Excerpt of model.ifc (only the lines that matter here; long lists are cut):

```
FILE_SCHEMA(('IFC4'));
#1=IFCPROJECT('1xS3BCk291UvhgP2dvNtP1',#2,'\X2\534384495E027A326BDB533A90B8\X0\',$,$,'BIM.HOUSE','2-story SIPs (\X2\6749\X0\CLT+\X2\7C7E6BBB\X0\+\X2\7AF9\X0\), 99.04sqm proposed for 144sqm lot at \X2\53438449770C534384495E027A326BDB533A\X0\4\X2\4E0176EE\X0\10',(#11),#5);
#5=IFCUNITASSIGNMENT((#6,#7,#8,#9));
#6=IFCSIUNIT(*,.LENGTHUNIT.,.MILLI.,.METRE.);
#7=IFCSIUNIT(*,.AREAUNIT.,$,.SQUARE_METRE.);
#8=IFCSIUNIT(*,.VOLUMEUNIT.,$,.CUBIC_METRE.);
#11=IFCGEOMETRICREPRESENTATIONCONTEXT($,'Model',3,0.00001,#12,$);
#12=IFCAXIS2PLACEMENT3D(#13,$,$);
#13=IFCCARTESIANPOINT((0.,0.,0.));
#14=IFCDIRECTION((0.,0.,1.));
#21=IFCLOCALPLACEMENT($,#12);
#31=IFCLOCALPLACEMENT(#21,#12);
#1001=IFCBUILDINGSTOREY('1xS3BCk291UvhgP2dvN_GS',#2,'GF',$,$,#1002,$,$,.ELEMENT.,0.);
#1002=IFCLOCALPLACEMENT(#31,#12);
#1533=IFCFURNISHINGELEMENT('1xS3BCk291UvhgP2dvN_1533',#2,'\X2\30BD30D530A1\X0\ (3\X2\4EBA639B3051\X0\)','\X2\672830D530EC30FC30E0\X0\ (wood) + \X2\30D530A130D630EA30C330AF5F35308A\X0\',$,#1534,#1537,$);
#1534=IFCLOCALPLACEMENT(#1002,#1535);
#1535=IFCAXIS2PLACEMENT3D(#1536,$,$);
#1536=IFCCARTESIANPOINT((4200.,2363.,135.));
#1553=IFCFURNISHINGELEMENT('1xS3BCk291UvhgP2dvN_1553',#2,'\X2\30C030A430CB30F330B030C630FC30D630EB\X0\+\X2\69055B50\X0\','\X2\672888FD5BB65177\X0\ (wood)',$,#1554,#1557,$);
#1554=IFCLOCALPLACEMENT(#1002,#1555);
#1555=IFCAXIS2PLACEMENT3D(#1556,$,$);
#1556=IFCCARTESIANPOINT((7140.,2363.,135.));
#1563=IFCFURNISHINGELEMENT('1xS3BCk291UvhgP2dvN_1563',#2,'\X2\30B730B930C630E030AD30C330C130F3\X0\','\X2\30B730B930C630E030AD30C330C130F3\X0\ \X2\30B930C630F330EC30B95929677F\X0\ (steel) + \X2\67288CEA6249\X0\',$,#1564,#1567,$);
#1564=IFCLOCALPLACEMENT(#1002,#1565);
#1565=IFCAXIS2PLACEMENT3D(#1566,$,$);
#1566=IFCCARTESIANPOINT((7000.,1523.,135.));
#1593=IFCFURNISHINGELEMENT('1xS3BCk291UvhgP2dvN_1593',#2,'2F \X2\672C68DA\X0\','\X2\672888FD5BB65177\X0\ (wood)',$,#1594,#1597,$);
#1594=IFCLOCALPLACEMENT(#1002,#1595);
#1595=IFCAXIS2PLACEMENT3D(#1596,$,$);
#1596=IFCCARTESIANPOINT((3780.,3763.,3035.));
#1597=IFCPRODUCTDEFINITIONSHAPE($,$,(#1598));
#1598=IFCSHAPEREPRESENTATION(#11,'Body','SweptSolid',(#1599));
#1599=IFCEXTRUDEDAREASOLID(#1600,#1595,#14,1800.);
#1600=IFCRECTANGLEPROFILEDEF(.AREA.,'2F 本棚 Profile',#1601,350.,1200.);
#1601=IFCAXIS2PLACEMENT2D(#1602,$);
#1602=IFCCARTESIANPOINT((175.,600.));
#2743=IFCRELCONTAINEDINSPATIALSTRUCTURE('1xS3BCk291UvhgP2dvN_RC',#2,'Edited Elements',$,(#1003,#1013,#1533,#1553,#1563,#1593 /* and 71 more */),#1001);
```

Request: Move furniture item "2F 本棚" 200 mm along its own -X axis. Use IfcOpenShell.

```python
import ifcopenshell
import ifcopenshell.api.geometry
import ifcopenshell.util.placement

model = ifcopenshell.open("model.ifc")

item = model.by_guid("1xS3BCk291UvhgP2dvN_1593")
matrix = ifcopenshell.util.placement.get_local_placement(item.ObjectPlacement)
matrix[:3, 3] -= matrix[:3, 0] * 200.0
ifcopenshell.api.geometry.edit_object_placement(model, product=item, matrix=matrix, is_si=False)

print(ifcopenshell.util.placement.get_local_placement(item.ObjectPlacement).round(3) + 0.0)

model.write("model_updated.ifc")
```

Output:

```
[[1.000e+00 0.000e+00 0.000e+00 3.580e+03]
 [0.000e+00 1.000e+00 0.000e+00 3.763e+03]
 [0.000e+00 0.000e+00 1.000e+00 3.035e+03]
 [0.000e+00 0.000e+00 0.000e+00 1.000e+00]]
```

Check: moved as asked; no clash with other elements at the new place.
